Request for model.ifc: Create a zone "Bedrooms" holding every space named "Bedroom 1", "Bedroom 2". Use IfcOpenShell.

First a look at what the model holds.

```python
import ifcopenshell

model = ifcopenshell.open("model.ifc")
print(model.schema)
seen = {}
for space in model.by_type("IfcSpace"):
    seen[space.LongName] = seen.get(space.LongName, 0) + 1
for name, count in sorted(seen.items(), key=str):
    print(count, "x", name)
print("zones:", [z.Name for z in model.by_type("IfcZone")][:20])
```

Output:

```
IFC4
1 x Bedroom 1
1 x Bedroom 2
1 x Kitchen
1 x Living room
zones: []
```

```python
import ifcopenshell
import ifcopenshell.api.group
import ifcopenshell.api.root

model = ifcopenshell.open("model.ifc")

names = {"Bedroom 1", "Bedroom 2"}
spaces = [s for s in model.by_type("IfcSpace") if s.LongName in names]

zone = ifcopenshell.api.root.create_entity(model, ifc_class="IfcZone", name="Bedrooms")
ifcopenshell.api.group.assign_group(model, products=spaces, group=zone)
print(len(spaces), "spaces in", zone.Name)

model.write("model_updated.ifc")
```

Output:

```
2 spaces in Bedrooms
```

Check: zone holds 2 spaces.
